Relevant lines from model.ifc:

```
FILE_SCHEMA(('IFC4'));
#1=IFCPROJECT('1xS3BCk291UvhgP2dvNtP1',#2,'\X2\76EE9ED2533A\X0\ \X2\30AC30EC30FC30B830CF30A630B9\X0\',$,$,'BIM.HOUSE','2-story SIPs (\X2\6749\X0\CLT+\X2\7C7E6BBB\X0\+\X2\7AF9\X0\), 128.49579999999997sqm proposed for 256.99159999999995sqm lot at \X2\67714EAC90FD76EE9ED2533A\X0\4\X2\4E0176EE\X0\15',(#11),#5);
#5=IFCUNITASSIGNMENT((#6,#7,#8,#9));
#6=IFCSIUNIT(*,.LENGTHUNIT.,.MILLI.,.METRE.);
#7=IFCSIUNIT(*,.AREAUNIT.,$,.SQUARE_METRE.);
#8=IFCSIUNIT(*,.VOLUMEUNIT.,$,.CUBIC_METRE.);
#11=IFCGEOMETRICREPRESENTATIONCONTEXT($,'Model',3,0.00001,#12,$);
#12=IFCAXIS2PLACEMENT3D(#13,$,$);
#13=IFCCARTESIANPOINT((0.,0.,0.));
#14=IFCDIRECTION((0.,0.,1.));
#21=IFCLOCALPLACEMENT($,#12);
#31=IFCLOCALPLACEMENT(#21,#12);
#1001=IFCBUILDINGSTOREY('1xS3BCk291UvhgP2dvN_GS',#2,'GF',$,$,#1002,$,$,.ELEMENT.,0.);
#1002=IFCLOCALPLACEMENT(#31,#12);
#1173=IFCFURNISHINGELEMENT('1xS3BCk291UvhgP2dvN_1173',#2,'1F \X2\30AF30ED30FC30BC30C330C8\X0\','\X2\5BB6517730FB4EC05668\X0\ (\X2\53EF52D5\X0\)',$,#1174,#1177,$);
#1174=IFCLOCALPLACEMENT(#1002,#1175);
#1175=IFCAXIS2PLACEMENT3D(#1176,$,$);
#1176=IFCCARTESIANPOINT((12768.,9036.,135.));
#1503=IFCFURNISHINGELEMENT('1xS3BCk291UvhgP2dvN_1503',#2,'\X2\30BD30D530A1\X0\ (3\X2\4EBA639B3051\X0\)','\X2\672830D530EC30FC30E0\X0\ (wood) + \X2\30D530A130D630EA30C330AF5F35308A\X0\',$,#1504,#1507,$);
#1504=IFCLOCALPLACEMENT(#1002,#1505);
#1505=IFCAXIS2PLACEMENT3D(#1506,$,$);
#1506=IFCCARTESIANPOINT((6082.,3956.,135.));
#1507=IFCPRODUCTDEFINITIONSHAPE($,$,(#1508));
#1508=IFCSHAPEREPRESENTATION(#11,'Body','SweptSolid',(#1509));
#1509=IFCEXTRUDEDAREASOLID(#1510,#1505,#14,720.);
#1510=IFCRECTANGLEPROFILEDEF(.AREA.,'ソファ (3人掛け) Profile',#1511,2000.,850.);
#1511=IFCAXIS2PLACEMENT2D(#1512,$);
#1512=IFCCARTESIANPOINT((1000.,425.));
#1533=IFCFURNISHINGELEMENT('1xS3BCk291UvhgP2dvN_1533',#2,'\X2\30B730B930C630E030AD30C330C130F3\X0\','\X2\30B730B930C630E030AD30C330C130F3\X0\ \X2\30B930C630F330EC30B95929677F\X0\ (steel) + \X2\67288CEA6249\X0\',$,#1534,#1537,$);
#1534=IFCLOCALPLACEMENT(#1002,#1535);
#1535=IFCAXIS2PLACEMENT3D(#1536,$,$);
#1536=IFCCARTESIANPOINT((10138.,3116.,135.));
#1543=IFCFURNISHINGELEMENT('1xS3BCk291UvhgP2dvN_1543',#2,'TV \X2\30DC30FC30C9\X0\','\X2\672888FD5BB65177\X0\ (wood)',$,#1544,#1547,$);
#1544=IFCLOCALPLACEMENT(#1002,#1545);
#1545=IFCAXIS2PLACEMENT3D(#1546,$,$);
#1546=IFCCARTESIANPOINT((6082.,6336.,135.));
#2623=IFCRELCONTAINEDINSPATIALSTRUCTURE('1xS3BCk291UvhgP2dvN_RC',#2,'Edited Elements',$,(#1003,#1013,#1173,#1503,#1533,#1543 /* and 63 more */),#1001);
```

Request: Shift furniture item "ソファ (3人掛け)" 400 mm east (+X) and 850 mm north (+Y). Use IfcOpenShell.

```python
import ifcopenshell
import ifcopenshell.api.geometry
import ifcopenshell.util.placement
import ifcopenshell.util.unit

model = ifcopenshell.open("model.ifc")
unit_scale = ifcopenshell.util.unit.calculate_unit_scale(model)

item = model.by_guid("1xS3BCk291UvhgP2dvN_1503")
matrix = ifcopenshell.util.placement.get_local_placement(item.ObjectPlacement)
matrix[0, 3] += 0.4 / unit_scale
matrix[1, 3] += 0.85 / unit_scale
ifcopenshell.api.geometry.edit_object_placement(model, product=item, matrix=matrix, is_si=False)

print(ifcopenshell.util.placement.get_local_placement(item.ObjectPlacement).round(3) + 0.0)

model.write("model_rev.ifc")
```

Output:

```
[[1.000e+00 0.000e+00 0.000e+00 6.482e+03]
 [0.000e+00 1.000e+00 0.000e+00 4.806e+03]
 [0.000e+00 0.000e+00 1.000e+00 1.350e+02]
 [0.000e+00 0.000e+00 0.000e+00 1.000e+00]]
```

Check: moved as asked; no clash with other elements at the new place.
